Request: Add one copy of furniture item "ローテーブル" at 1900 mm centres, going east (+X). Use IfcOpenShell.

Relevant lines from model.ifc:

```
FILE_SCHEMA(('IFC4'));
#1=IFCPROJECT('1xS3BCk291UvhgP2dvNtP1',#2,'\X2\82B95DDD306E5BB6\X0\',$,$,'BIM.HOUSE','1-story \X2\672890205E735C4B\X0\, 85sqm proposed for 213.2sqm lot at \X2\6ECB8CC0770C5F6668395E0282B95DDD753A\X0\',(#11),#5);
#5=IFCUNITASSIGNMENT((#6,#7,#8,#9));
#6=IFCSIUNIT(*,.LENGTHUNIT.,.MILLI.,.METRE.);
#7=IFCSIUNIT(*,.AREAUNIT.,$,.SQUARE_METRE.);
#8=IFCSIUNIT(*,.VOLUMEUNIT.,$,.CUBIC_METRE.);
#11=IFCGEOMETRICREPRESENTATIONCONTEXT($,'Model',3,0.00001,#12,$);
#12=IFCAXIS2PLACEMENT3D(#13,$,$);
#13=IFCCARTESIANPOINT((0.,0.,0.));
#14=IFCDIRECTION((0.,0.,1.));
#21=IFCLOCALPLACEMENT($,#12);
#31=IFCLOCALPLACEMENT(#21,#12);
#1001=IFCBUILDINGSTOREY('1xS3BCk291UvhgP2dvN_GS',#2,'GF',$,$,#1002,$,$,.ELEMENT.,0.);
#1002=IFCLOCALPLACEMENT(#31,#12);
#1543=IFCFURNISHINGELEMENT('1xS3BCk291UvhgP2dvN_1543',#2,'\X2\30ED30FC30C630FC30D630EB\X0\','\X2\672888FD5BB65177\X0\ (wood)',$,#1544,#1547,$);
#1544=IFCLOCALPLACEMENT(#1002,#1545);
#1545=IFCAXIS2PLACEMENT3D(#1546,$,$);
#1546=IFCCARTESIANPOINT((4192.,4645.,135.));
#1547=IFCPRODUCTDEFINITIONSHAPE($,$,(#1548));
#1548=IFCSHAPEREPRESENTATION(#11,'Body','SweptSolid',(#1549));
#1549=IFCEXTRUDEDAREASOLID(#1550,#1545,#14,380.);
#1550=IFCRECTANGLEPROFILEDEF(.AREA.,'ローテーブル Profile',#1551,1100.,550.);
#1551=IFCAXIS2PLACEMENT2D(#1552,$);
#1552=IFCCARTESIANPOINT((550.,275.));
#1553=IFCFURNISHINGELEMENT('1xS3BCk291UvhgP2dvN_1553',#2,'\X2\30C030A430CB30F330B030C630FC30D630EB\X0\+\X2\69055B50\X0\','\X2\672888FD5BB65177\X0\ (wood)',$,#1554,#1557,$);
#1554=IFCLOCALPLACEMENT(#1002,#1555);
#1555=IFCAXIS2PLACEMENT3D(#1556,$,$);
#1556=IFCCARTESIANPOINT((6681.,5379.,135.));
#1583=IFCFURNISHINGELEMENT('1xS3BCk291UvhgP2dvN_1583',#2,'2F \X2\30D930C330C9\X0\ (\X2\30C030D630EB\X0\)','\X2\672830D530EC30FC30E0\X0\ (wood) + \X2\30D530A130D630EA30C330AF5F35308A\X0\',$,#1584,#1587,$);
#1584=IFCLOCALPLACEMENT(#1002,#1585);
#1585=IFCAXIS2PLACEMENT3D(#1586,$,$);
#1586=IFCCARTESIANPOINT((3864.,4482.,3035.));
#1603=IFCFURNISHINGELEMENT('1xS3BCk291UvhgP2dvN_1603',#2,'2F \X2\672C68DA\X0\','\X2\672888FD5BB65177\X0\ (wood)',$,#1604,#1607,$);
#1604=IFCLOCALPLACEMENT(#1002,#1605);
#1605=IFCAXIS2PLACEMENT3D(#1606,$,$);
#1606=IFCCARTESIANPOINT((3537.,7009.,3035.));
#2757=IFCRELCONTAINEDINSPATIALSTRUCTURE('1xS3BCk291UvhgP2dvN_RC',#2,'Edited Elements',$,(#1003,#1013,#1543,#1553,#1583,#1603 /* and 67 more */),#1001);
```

```python
import numpy as np
import ifcopenshell
import ifcopenshell.api.geometry
import ifcopenshell.api.root
import ifcopenshell.util.element
import ifcopenshell.util.placement
import ifcopenshell.util.unit

model = ifcopenshell.open("model.ifc")
unit_scale = ifcopenshell.util.unit.calculate_unit_scale(model)


def reuse_history(source, copy):
    """copy_class also copies each property set's owner history, people and application; keep the originals."""
    for rel in copy.IsDefinedBy:
        if rel.is_a("IfcRelDefinesByProperties") and (history := rel.RelatingPropertyDefinition.OwnerHistory):
            rel.RelatingPropertyDefinition.OwnerHistory = source.OwnerHistory
            ifcopenshell.util.element.remove_deep2(model, history)


source = model.by_guid("1xS3BCk291UvhgP2dvN_1543")
base = ifcopenshell.util.placement.get_local_placement(source.ObjectPlacement)
step = np.array([1.0, 0.0, 0.0]) * 1.9 / unit_scale

for i in range(1, 2):
    copy = ifcopenshell.api.root.copy_class(model, product=source)
    copy.Representation = ifcopenshell.util.element.copy_deep(
        model, source.Representation, exclude=["IfcGeometricRepresentationContext", "IfcRepresentationMap"]
    )
    reuse_history(source, copy)
    matrix = base.copy()
    matrix[:3, 3] += i * step
    print("added at", matrix[:3, 3].round(3) + 0.0)
    ifcopenshell.api.geometry.edit_object_placement(model, product=copy, matrix=matrix, is_si=False)

model.write("model-out.ifc")
```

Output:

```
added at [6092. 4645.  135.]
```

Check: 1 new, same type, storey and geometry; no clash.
